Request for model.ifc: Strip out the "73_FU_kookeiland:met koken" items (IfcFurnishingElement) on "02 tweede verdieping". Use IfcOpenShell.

First a look at what the model holds.

```python
import ifcopenshell
import ifcopenshell.util.element

model = ifcopenshell.open("model.ifc")
print(model.schema)
storey = next(s for s in model.by_type("IfcBuildingStorey") if s.Name == "02 tweede verdieping")
furniture = [e for e in ifcopenshell.util.element.get_decomposition(storey) if e.is_a("IfcFurnishingElement")]
seen = {}
for e in furniture:
    element_type = ifcopenshell.util.element.get_type(e)
    name = element_type.Name if element_type not in (None, e) else None
    seen[name] = seen.get(name, 0) + 1
for name, count in sorted(seen.items(), key=str):
    print(count, "x", name)
```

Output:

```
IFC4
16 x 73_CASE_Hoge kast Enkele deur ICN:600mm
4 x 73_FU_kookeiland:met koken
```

```python
import ifcopenshell
import ifcopenshell.api.root
import ifcopenshell.util.element

model = ifcopenshell.open("model.ifc")

storey = next(s for s in model.by_type("IfcBuildingStorey") if s.Name == "02 tweede verdieping")
furniture = [e for e in ifcopenshell.util.element.get_decomposition(storey) if e.is_a("IfcFurnishingElement")]
targets = [e for e in furniture if (t := ifcopenshell.util.element.get_type(e)) not in (None, e) and t.Name == "73_FU_kookeiland:met koken"]

for e in targets:
    ifcopenshell.api.root.remove_product(model, product=e)
print(len(targets), "removed")

model.write("model_rev.ifc")
```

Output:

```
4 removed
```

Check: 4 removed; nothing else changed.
